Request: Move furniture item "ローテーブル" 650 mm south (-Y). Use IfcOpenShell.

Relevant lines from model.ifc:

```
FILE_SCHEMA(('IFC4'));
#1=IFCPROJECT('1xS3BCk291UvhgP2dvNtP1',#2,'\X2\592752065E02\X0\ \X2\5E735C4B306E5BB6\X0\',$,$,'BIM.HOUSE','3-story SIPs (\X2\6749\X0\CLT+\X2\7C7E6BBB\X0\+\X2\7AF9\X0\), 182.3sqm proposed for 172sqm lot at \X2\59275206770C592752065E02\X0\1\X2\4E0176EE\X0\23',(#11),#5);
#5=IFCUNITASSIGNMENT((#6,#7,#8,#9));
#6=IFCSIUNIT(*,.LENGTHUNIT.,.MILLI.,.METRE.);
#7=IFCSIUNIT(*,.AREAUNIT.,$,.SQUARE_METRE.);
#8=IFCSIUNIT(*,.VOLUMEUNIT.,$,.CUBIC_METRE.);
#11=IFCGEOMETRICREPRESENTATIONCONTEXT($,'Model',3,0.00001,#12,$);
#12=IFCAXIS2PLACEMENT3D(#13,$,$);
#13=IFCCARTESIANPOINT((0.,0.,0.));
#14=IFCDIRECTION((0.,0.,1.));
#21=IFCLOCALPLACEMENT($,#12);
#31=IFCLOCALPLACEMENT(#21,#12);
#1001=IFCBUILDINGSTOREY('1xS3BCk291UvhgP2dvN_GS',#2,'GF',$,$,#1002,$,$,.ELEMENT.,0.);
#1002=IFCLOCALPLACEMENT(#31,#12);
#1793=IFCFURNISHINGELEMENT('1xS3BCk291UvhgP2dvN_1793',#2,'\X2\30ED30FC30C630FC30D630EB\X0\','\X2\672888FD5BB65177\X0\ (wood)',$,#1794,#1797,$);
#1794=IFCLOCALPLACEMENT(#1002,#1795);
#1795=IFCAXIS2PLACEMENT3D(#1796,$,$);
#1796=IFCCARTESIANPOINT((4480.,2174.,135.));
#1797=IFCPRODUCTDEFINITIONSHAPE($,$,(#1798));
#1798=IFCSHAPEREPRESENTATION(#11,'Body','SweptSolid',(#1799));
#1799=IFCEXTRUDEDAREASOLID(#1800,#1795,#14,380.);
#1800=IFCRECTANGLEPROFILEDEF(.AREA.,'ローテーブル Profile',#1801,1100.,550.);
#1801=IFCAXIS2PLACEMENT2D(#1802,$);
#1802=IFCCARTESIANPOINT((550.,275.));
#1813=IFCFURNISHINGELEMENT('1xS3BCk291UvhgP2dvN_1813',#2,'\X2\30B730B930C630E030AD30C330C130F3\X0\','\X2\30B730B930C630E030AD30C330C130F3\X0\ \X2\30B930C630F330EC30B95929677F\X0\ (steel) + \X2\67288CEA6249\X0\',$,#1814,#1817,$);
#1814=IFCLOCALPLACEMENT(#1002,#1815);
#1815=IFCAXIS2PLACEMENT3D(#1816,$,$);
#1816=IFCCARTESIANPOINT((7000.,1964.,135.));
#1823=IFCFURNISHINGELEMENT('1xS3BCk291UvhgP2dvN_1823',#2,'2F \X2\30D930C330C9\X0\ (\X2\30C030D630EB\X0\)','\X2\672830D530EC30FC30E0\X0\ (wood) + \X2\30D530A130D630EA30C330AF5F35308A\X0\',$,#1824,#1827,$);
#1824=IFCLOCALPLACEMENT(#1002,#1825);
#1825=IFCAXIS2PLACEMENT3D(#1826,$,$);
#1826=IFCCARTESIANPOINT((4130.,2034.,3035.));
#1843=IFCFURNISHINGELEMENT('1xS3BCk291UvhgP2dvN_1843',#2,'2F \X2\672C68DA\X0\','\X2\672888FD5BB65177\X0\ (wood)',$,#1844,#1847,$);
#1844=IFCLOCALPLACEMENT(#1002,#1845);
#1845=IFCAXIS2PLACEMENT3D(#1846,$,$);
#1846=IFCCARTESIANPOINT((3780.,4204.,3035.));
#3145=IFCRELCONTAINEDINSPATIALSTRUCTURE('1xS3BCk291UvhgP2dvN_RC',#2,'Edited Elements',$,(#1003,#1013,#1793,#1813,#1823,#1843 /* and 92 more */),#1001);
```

```python
import ifcopenshell
import ifcopenshell.api.geometry
import ifcopenshell.util.placement

model = ifcopenshell.open("model.ifc")

item = model.by_guid("1xS3BCk291UvhgP2dvN_1793")
matrix = ifcopenshell.util.placement.get_local_placement(item.ObjectPlacement)
matrix[1, 3] -= 650.0
ifcopenshell.api.geometry.edit_object_placement(model, product=item, matrix=matrix, is_si=False)

print(ifcopenshell.util.placement.get_local_placement(item.ObjectPlacement).round(3) + 0.0)

model.write("model-out.ifc")
```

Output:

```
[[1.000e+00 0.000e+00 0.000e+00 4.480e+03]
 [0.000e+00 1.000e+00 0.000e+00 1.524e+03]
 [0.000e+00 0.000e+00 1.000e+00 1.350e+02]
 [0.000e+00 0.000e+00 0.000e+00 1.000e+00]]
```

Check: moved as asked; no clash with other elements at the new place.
